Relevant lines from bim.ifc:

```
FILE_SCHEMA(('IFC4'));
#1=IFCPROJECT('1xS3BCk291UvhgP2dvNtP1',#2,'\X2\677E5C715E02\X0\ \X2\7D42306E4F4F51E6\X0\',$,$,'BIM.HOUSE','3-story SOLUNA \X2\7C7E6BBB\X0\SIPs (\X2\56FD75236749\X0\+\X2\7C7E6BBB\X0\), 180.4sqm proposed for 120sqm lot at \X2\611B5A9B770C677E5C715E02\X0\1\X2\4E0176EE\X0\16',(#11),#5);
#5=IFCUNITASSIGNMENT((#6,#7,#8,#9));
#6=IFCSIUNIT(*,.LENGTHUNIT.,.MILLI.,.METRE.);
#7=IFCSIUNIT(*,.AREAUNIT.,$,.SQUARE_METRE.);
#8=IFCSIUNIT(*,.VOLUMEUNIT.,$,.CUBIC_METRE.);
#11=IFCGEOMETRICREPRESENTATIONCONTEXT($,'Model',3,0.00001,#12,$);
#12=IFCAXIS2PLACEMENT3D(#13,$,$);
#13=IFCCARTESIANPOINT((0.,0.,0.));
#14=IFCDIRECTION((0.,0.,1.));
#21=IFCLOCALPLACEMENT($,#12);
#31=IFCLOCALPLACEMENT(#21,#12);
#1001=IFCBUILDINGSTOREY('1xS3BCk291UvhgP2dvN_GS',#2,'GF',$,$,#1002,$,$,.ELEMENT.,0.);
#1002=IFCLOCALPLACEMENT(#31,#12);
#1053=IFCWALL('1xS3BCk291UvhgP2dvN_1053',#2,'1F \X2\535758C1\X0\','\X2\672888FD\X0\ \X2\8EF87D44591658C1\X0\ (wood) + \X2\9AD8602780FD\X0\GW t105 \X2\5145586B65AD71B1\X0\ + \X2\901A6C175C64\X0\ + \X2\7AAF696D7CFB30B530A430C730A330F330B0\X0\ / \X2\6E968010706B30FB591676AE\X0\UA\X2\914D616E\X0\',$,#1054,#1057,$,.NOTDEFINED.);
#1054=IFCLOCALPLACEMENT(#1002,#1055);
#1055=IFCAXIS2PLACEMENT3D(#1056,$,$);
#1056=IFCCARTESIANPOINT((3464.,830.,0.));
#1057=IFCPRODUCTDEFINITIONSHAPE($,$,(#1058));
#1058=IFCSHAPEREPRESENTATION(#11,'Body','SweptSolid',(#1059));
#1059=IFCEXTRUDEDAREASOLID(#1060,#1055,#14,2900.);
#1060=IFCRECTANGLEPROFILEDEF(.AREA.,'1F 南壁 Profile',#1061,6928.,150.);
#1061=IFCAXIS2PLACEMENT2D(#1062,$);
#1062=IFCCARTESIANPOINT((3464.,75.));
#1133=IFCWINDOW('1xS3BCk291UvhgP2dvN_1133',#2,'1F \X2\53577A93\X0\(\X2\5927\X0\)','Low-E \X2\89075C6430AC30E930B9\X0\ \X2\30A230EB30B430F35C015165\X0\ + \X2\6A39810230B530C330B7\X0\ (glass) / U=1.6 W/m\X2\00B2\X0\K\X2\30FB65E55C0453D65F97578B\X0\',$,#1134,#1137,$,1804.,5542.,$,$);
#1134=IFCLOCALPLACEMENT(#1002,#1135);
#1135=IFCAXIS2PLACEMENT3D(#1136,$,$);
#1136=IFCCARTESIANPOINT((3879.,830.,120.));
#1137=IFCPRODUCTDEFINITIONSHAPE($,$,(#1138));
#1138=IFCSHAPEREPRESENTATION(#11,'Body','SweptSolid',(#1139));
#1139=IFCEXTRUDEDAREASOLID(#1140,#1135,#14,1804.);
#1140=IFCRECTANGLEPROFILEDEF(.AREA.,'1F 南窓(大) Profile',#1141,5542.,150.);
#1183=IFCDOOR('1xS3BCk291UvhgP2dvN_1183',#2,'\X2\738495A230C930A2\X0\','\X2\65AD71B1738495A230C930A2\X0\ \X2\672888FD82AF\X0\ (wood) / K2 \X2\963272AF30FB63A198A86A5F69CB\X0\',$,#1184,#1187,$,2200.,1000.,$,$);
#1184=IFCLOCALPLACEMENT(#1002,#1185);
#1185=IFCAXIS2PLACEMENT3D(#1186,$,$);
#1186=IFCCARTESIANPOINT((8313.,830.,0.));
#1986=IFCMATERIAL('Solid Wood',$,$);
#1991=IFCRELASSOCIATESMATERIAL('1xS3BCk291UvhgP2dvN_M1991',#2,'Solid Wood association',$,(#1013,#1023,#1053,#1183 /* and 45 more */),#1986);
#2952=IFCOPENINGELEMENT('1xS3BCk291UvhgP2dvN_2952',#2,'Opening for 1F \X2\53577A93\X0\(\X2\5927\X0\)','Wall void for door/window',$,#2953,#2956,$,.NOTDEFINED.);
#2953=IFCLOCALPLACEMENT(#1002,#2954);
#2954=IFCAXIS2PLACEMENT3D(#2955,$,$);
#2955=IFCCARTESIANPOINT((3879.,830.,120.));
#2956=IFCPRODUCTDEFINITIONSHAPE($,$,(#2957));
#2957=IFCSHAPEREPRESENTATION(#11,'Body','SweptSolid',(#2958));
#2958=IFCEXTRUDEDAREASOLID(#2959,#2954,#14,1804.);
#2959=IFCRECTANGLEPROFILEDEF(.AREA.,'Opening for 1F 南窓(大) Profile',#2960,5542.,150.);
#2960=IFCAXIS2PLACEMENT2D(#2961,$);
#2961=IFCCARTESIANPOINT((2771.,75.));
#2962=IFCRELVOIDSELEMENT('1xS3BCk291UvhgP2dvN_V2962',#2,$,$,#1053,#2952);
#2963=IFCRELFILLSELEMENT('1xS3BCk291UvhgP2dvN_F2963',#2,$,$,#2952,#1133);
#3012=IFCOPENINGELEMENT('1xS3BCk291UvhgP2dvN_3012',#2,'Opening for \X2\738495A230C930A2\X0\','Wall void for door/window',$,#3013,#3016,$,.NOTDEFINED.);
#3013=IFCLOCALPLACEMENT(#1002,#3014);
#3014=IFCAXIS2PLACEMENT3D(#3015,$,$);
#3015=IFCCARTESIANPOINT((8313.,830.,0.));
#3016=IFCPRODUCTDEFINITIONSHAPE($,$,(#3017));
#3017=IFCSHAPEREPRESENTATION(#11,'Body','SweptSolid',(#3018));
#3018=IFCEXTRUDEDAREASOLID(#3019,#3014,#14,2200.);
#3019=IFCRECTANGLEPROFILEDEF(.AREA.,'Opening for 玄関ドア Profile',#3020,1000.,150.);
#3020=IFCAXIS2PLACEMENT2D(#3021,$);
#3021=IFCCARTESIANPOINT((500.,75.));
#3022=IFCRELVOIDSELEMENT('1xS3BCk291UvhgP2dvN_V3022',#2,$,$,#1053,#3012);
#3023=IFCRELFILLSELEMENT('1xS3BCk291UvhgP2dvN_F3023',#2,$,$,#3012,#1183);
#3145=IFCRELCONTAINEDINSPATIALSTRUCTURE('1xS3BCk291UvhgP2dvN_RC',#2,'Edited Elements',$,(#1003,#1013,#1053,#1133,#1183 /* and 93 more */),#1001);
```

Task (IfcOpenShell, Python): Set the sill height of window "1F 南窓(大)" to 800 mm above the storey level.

```python
import numpy as np
import ifcopenshell
import ifcopenshell.api.geometry
import ifcopenshell.geom
import ifcopenshell.util.element
import ifcopenshell.util.placement
import ifcopenshell.util.shape
import ifcopenshell.util.unit

model = ifcopenshell.open("bim.ifc")
unit_scale = ifcopenshell.util.unit.calculate_unit_scale(model)

window = model.by_id(1133)
opening = window.FillsVoids[0].RelatingOpeningElement
storey = ifcopenshell.util.element.get_container(window, ifc_class="IfcBuildingStorey")
level = ifcopenshell.util.placement.get_local_placement(storey.ObjectPlacement)[2, 3]

# The opening's origin need not be at the sill, so measure its lowest point.
shape = ifcopenshell.geom.create_shape(ifcopenshell.geom.settings(), opening)
bottom = ifcopenshell.util.shape.get_shape_bottom_elevation(shape, shape.geometry) / unit_scale
dz = level + 0.8 / unit_scale - bottom

shift = np.array([0.0, 0.0, dz])
# The window is not placed relative to its opening, so move both.
for product in (opening, window):
    matrix = ifcopenshell.util.placement.get_local_placement(product.ObjectPlacement)
    matrix[:3, 3] += shift
    ifcopenshell.api.geometry.edit_object_placement(model, product=product, matrix=matrix, is_si=False)

print(f"moved by {dz * unit_scale:+.3f} m")

model.write("bim-out.ifc")
```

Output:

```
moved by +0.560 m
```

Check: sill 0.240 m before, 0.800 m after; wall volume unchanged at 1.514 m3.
